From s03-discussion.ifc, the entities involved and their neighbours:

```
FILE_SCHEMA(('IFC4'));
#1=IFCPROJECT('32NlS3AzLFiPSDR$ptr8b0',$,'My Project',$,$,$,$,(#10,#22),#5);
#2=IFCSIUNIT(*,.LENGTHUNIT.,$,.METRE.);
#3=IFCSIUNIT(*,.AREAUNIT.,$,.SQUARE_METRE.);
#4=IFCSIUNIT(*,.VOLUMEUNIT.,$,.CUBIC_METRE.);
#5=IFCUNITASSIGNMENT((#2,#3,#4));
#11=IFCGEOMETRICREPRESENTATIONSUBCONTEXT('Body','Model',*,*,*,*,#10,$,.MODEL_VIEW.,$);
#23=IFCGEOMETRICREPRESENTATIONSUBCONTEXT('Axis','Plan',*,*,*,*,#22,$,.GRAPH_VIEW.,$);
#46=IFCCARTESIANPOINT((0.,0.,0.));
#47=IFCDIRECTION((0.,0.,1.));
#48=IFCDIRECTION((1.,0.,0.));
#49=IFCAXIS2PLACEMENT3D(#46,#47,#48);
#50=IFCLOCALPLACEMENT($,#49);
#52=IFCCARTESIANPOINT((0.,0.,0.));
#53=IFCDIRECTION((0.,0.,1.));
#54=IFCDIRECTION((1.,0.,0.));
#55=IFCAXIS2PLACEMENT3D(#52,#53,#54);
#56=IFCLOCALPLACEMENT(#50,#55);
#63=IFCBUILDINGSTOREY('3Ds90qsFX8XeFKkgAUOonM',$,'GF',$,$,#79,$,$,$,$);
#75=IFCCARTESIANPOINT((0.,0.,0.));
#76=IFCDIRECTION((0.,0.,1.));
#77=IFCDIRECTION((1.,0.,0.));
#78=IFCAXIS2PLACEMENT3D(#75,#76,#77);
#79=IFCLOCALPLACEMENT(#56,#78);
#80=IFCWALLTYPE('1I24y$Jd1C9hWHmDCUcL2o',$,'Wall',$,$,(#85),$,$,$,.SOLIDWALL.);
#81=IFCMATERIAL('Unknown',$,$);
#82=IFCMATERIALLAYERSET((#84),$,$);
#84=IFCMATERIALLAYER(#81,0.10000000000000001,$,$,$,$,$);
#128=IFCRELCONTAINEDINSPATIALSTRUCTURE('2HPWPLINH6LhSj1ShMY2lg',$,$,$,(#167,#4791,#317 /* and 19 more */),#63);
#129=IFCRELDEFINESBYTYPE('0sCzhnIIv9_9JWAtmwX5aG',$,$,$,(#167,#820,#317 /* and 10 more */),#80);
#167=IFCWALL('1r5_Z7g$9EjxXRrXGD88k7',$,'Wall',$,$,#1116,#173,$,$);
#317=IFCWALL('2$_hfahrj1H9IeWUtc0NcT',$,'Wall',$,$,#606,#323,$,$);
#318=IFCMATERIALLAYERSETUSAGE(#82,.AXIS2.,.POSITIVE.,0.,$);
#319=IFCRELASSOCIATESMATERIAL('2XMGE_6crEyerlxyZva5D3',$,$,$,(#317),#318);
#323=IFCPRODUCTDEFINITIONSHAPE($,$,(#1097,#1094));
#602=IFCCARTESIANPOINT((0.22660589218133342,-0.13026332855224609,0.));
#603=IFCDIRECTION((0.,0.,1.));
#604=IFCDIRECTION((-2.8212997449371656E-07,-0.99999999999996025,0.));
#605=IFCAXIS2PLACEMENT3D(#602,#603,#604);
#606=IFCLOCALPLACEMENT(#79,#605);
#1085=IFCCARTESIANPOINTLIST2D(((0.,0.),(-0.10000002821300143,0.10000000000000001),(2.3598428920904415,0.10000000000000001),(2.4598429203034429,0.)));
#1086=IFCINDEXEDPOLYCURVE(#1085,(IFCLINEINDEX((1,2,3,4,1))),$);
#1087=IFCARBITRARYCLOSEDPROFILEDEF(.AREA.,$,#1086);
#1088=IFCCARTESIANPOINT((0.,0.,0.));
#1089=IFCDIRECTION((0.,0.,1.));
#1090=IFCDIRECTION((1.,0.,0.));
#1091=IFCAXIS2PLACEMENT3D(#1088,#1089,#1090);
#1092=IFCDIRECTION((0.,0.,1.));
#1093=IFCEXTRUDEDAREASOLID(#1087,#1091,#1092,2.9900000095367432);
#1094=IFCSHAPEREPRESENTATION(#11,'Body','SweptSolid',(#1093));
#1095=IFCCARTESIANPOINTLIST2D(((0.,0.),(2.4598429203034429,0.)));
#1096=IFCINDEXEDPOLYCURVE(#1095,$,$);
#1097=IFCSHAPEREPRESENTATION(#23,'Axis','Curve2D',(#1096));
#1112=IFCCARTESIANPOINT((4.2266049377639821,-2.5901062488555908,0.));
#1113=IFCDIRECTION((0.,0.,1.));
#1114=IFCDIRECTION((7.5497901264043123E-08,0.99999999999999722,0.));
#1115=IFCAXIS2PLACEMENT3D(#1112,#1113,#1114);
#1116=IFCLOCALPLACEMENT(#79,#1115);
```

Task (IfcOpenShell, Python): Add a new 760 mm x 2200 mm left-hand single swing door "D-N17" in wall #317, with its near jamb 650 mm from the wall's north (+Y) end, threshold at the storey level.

```python
import numpy as np
import ifcopenshell
import ifcopenshell.api.feature
import ifcopenshell.api.geometry
import ifcopenshell.api.root
import ifcopenshell.api.spatial
import ifcopenshell.geom
import ifcopenshell.util.element
import ifcopenshell.util.placement
import ifcopenshell.util.representation
import ifcopenshell.util.shape
import ifcopenshell.util.unit

model = ifcopenshell.open("s03-discussion.ifc")
unit_scale = ifcopenshell.util.unit.calculate_unit_scale(model)
settings = ifcopenshell.geom.settings()


def volume(element):
    """Net volume in cubic metres, openings subtracted."""
    shape = ifcopenshell.geom.create_shape(settings, element)
    return ifcopenshell.util.shape.get_volume(shape.geometry)


wall = model.by_id(317)
storey = ifcopenshell.util.element.get_container(wall, ifc_class="IfcBuildingStorey")
context = ifcopenshell.util.representation.get_context(model, "Model", "Body", "MODEL_VIEW")
before = volume(wall)

width, height, from_end, sill = 0.76, 2.2, 0.65, 0.0  # metres

# The wall runs along its own X axis, and the end named is its -X end.
wall_shape = ifcopenshell.geom.create_shape(settings, wall)
x, y, z = ifcopenshell.util.shape.get_vertices(wall_shape.geometry).T
start = x.min() + from_end
face, thickness = float(y.min()), float(y.max() - y.min())
wall_matrix = ifcopenshell.util.placement.get_local_placement(wall.ObjectPlacement)
level = ifcopenshell.util.placement.get_local_placement(storey.ObjectPlacement)[2, 3]


def in_wall(x, y):
    """Placement at x, y metres in the wall's axes, at sill height."""
    matrix = wall_matrix.copy()
    matrix[:, 3] = wall_matrix @ np.array([x / unit_scale, y / unit_scale, 0.0, 1.0])
    matrix[2, 3] = level + sill / unit_scale
    return matrix


# Opening: a box that overshoots both wall faces by 50 mm.
opening = ifcopenshell.api.root.create_entity(model, ifc_class="IfcOpeningElement", predefined_type="OPENING")
box = ifcopenshell.api.geometry.add_wall_representation(
    model, context=context, length=width, height=height, thickness=thickness + 0.1
)
ifcopenshell.api.geometry.assign_representation(model, product=opening, representation=box)
ifcopenshell.api.geometry.edit_object_placement(model, product=opening, matrix=in_wall(start, face - 0.05), is_si=False)
ifcopenshell.api.feature.add_feature(model, feature=opening, element=wall)

door = ifcopenshell.api.root.create_entity(model, ifc_class="IfcDoor", name="D-N17", predefined_type="DOOR")
door.OverallWidth, door.OverallHeight = width / unit_scale, height / unit_scale
door.OperationType = "SINGLE_SWING_LEFT"
body = ifcopenshell.api.geometry.add_door_representation(
    model,
    context=context,
    overall_width=door.OverallWidth,
    overall_height=door.OverallHeight,
    operation_type="SINGLE_SWING_LEFT",
    lining_properties={"LiningDepth": thickness / unit_scale, "ThresholdDepth": thickness / unit_scale},
)
ifcopenshell.api.geometry.assign_representation(model, product=door, representation=body)
ifcopenshell.api.spatial.assign_container(model, products=[door], relating_structure=storey)
ifcopenshell.api.feature.add_filling(model, opening=opening, element=door)

# The lining spans the wall, so the door starts at the wall face.
ifcopenshell.api.geometry.edit_object_placement(model, product=door, matrix=in_wall(start, face), is_si=False)

after = volume(wall)

print(f"wall volume {before:.3f} -> {after:.3f} m3")

model.write("s03-discussion_edited.ifc")
```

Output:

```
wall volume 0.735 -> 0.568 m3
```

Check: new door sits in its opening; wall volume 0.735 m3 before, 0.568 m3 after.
